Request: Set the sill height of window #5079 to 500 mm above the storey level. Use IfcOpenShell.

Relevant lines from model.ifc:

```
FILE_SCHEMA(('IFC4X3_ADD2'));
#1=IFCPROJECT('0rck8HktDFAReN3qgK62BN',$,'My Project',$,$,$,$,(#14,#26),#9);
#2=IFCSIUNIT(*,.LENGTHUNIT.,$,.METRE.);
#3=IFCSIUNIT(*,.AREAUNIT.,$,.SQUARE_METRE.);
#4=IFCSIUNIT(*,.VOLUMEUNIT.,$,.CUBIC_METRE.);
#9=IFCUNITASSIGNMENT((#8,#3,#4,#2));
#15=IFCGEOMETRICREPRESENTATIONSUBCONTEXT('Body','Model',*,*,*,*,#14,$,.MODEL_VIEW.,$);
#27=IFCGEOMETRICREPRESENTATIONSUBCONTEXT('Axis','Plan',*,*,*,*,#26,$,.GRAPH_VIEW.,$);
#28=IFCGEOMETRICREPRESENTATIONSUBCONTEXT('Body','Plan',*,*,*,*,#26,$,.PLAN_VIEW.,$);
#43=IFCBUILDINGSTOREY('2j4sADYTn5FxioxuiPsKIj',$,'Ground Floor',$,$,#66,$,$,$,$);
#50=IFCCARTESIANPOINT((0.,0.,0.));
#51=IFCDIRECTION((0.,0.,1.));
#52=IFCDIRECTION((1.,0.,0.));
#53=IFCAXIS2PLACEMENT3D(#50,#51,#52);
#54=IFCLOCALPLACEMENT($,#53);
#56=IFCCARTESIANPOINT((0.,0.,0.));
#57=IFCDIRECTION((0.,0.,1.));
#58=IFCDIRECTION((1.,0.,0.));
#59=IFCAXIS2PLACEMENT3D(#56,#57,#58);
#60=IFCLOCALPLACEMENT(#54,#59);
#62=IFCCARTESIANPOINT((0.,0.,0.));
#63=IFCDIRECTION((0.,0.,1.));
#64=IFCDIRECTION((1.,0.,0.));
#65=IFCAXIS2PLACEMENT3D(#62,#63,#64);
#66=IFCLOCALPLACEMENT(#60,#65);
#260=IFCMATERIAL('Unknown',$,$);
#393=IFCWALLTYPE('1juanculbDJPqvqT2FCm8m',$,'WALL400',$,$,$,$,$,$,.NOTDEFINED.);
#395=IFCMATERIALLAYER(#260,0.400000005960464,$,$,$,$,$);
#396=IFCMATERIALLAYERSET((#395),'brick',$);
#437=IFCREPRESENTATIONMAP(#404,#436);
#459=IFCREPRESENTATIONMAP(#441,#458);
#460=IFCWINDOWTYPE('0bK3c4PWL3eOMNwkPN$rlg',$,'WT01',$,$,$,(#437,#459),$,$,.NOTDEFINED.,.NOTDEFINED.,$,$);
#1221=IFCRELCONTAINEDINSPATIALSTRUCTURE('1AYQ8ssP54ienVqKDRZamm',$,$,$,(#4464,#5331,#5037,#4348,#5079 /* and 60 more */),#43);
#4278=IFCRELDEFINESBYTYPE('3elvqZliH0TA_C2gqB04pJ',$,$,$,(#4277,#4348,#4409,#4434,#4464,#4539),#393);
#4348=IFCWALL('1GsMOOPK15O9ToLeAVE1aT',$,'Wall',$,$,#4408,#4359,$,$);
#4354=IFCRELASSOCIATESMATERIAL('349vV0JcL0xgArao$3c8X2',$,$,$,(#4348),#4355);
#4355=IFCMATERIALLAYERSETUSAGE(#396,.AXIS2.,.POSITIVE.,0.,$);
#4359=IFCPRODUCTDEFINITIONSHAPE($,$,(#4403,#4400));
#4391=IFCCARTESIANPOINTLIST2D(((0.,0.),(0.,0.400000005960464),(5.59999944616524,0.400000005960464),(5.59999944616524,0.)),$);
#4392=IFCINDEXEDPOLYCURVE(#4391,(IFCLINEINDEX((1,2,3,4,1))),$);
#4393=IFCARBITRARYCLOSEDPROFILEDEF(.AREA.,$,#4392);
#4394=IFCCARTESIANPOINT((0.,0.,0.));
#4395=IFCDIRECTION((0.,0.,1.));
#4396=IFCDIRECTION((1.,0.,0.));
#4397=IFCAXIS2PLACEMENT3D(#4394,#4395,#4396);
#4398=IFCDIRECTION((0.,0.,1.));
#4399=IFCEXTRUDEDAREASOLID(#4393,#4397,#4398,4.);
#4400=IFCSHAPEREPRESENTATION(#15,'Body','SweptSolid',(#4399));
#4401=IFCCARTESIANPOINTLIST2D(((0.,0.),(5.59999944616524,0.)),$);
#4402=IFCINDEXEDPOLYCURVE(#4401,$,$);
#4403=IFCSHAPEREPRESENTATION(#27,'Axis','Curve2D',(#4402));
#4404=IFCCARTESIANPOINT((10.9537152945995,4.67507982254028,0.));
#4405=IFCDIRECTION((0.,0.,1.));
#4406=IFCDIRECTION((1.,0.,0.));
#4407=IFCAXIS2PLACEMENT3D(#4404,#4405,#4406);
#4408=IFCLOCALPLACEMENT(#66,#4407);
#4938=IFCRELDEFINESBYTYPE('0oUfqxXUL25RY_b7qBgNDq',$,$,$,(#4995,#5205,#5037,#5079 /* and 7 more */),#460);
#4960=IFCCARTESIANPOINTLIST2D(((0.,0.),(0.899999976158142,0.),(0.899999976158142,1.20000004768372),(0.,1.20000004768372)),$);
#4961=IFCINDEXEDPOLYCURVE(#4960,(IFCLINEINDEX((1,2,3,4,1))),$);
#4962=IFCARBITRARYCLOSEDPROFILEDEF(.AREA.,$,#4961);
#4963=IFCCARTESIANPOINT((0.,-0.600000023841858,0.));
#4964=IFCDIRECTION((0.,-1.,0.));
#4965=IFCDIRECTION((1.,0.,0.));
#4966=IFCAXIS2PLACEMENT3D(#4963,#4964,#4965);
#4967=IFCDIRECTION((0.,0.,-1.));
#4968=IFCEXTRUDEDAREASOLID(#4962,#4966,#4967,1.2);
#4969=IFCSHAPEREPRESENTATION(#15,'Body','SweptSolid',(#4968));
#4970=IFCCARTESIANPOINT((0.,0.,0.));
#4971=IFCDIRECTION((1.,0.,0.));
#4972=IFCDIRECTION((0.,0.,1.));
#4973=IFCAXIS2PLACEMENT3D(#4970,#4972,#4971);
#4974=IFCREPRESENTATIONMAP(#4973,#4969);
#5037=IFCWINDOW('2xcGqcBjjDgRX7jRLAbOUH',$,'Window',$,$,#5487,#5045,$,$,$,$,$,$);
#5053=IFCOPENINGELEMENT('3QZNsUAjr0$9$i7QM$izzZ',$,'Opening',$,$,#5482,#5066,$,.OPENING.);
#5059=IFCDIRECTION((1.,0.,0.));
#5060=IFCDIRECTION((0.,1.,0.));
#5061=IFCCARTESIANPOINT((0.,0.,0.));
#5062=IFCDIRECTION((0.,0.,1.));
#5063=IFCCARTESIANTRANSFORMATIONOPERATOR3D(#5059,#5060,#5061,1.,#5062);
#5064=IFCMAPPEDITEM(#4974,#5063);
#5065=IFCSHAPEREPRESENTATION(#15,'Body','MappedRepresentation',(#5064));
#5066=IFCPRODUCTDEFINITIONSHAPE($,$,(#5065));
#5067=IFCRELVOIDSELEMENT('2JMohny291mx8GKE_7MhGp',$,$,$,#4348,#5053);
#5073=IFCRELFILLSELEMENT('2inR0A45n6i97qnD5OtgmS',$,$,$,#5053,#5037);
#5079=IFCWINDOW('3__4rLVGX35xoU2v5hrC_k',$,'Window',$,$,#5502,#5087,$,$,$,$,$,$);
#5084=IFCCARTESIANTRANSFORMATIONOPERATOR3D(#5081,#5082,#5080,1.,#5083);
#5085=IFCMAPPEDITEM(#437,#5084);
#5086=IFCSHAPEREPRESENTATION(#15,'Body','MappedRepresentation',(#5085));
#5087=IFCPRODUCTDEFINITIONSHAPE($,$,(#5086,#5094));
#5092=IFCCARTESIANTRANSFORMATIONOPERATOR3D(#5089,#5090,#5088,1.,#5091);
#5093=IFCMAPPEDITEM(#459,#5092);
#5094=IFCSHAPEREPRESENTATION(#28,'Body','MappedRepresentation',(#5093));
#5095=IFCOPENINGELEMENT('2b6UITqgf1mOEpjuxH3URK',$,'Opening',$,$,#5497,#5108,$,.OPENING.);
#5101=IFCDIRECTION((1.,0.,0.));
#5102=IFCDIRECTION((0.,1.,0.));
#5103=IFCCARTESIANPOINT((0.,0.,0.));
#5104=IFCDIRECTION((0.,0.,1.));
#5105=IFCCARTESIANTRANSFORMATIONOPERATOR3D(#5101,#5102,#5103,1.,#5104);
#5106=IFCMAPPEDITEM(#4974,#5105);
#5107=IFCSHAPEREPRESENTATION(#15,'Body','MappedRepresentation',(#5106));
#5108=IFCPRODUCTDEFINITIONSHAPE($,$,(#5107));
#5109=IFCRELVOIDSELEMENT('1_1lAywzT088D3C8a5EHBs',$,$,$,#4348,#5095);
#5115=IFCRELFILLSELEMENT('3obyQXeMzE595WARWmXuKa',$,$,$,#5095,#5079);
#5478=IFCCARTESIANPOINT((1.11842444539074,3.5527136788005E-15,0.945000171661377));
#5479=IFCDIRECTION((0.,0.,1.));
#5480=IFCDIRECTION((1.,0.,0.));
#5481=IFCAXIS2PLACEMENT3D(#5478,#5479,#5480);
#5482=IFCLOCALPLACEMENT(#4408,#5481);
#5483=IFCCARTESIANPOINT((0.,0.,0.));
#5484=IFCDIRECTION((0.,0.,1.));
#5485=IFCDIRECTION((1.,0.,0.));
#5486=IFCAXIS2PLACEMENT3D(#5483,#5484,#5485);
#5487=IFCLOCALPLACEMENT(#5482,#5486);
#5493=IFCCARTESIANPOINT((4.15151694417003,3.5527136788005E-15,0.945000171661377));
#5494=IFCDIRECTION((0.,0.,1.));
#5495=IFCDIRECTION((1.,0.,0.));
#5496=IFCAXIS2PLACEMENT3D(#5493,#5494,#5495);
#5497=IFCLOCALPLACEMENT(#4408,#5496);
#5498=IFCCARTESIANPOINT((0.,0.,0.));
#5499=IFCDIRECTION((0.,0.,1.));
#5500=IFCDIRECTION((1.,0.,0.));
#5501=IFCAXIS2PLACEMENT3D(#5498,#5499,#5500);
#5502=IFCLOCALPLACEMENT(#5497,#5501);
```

```python
import numpy as np
import ifcopenshell
import ifcopenshell.api.geometry
import ifcopenshell.geom
import ifcopenshell.util.element
import ifcopenshell.util.placement
import ifcopenshell.util.shape
import ifcopenshell.util.unit

model = ifcopenshell.open("model.ifc")
unit_scale = ifcopenshell.util.unit.calculate_unit_scale(model)

window = model.by_guid("3__4rLVGX35xoU2v5hrC_k")
opening = window.FillsVoids[0].RelatingOpeningElement
storey = ifcopenshell.util.element.get_container(window, ifc_class="IfcBuildingStorey")
level = ifcopenshell.util.placement.get_local_placement(storey.ObjectPlacement)[2, 3]

# The opening's origin need not be at the sill, so measure its lowest point.
shape = ifcopenshell.geom.create_shape(ifcopenshell.geom.settings(), opening)
bottom = ifcopenshell.util.shape.get_shape_bottom_elevation(shape, shape.geometry) / unit_scale
dz = level + 0.5 - bottom

shift = np.array([0.0, 0.0, dz])
# The window is placed relative to its opening, so it follows when the opening moves.
matrix = ifcopenshell.util.placement.get_local_placement(opening.ObjectPlacement)
matrix[:3, 3] += shift
ifcopenshell.api.geometry.edit_object_placement(
    model, product=opening, matrix=matrix, is_si=False, should_transform_children=True
)

print(f"moved by {dz * unit_scale:+.3f} m")

model.write("model_edited.ifc")
```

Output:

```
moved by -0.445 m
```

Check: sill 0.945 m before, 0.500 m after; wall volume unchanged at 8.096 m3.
